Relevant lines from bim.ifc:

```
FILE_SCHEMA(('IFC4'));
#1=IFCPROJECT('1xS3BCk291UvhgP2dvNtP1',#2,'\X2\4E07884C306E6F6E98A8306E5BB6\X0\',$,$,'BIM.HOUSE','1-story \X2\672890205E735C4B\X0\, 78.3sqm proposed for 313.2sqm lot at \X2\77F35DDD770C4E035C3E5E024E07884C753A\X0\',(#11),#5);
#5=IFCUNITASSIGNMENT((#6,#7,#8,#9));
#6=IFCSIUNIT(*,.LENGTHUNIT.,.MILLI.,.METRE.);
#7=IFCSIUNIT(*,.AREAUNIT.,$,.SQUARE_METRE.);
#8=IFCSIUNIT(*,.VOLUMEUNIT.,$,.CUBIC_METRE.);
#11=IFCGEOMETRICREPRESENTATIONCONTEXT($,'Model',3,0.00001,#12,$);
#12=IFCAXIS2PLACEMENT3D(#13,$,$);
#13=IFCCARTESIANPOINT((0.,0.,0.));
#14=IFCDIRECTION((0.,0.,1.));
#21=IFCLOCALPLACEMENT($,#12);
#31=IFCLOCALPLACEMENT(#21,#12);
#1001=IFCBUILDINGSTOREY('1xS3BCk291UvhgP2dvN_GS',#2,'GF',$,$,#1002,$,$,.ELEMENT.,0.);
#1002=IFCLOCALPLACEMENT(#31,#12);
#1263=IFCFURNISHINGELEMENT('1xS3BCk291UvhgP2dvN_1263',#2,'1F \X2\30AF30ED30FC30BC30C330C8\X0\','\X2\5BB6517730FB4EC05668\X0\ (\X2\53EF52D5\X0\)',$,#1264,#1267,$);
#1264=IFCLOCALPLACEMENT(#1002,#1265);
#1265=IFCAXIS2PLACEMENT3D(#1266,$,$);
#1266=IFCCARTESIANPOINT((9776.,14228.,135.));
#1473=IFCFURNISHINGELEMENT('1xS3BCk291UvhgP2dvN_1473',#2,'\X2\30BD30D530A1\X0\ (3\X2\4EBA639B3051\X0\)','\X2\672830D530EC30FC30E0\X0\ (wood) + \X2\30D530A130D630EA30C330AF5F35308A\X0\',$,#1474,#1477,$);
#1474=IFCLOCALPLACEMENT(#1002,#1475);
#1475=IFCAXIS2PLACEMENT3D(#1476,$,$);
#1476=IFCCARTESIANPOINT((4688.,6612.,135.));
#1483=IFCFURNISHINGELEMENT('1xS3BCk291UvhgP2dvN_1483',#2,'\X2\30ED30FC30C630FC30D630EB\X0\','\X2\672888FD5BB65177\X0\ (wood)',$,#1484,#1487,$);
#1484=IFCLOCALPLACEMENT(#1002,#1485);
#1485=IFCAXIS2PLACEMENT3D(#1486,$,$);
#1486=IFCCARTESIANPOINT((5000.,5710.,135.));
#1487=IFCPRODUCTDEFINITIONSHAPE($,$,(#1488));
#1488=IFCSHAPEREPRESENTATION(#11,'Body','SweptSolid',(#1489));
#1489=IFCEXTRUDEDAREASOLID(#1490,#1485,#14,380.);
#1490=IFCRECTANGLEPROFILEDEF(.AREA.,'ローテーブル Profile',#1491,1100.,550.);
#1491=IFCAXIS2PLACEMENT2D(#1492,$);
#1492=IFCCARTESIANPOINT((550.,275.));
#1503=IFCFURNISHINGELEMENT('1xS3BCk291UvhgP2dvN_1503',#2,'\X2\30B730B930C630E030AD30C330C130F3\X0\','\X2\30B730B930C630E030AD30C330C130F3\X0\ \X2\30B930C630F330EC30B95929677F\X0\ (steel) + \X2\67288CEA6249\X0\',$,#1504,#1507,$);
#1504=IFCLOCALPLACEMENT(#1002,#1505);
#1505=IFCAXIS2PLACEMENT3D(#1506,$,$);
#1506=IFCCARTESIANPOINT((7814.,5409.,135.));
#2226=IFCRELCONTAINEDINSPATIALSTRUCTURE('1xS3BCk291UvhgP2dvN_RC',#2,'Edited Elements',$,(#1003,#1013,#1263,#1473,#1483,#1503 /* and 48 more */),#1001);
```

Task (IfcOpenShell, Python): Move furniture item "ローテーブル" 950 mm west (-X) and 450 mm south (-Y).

```python
import ifcopenshell
import ifcopenshell.api.geometry
import ifcopenshell.util.placement
import ifcopenshell.util.unit

model = ifcopenshell.open("bim.ifc")
unit_scale = ifcopenshell.util.unit.calculate_unit_scale(model)

item = model.by_id(1483)
matrix = ifcopenshell.util.placement.get_local_placement(item.ObjectPlacement)
matrix[0, 3] -= 0.95 / unit_scale
matrix[1, 3] -= 0.45 / unit_scale
ifcopenshell.api.geometry.edit_object_placement(model, product=item, matrix=matrix, is_si=False)

print(ifcopenshell.util.placement.get_local_placement(item.ObjectPlacement).round(3) + 0.0)

model.write("bim_rev.ifc")
```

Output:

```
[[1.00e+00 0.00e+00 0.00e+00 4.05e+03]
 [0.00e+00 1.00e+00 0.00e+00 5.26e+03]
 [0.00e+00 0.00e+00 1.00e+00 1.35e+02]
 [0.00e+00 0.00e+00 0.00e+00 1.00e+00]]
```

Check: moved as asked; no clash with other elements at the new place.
